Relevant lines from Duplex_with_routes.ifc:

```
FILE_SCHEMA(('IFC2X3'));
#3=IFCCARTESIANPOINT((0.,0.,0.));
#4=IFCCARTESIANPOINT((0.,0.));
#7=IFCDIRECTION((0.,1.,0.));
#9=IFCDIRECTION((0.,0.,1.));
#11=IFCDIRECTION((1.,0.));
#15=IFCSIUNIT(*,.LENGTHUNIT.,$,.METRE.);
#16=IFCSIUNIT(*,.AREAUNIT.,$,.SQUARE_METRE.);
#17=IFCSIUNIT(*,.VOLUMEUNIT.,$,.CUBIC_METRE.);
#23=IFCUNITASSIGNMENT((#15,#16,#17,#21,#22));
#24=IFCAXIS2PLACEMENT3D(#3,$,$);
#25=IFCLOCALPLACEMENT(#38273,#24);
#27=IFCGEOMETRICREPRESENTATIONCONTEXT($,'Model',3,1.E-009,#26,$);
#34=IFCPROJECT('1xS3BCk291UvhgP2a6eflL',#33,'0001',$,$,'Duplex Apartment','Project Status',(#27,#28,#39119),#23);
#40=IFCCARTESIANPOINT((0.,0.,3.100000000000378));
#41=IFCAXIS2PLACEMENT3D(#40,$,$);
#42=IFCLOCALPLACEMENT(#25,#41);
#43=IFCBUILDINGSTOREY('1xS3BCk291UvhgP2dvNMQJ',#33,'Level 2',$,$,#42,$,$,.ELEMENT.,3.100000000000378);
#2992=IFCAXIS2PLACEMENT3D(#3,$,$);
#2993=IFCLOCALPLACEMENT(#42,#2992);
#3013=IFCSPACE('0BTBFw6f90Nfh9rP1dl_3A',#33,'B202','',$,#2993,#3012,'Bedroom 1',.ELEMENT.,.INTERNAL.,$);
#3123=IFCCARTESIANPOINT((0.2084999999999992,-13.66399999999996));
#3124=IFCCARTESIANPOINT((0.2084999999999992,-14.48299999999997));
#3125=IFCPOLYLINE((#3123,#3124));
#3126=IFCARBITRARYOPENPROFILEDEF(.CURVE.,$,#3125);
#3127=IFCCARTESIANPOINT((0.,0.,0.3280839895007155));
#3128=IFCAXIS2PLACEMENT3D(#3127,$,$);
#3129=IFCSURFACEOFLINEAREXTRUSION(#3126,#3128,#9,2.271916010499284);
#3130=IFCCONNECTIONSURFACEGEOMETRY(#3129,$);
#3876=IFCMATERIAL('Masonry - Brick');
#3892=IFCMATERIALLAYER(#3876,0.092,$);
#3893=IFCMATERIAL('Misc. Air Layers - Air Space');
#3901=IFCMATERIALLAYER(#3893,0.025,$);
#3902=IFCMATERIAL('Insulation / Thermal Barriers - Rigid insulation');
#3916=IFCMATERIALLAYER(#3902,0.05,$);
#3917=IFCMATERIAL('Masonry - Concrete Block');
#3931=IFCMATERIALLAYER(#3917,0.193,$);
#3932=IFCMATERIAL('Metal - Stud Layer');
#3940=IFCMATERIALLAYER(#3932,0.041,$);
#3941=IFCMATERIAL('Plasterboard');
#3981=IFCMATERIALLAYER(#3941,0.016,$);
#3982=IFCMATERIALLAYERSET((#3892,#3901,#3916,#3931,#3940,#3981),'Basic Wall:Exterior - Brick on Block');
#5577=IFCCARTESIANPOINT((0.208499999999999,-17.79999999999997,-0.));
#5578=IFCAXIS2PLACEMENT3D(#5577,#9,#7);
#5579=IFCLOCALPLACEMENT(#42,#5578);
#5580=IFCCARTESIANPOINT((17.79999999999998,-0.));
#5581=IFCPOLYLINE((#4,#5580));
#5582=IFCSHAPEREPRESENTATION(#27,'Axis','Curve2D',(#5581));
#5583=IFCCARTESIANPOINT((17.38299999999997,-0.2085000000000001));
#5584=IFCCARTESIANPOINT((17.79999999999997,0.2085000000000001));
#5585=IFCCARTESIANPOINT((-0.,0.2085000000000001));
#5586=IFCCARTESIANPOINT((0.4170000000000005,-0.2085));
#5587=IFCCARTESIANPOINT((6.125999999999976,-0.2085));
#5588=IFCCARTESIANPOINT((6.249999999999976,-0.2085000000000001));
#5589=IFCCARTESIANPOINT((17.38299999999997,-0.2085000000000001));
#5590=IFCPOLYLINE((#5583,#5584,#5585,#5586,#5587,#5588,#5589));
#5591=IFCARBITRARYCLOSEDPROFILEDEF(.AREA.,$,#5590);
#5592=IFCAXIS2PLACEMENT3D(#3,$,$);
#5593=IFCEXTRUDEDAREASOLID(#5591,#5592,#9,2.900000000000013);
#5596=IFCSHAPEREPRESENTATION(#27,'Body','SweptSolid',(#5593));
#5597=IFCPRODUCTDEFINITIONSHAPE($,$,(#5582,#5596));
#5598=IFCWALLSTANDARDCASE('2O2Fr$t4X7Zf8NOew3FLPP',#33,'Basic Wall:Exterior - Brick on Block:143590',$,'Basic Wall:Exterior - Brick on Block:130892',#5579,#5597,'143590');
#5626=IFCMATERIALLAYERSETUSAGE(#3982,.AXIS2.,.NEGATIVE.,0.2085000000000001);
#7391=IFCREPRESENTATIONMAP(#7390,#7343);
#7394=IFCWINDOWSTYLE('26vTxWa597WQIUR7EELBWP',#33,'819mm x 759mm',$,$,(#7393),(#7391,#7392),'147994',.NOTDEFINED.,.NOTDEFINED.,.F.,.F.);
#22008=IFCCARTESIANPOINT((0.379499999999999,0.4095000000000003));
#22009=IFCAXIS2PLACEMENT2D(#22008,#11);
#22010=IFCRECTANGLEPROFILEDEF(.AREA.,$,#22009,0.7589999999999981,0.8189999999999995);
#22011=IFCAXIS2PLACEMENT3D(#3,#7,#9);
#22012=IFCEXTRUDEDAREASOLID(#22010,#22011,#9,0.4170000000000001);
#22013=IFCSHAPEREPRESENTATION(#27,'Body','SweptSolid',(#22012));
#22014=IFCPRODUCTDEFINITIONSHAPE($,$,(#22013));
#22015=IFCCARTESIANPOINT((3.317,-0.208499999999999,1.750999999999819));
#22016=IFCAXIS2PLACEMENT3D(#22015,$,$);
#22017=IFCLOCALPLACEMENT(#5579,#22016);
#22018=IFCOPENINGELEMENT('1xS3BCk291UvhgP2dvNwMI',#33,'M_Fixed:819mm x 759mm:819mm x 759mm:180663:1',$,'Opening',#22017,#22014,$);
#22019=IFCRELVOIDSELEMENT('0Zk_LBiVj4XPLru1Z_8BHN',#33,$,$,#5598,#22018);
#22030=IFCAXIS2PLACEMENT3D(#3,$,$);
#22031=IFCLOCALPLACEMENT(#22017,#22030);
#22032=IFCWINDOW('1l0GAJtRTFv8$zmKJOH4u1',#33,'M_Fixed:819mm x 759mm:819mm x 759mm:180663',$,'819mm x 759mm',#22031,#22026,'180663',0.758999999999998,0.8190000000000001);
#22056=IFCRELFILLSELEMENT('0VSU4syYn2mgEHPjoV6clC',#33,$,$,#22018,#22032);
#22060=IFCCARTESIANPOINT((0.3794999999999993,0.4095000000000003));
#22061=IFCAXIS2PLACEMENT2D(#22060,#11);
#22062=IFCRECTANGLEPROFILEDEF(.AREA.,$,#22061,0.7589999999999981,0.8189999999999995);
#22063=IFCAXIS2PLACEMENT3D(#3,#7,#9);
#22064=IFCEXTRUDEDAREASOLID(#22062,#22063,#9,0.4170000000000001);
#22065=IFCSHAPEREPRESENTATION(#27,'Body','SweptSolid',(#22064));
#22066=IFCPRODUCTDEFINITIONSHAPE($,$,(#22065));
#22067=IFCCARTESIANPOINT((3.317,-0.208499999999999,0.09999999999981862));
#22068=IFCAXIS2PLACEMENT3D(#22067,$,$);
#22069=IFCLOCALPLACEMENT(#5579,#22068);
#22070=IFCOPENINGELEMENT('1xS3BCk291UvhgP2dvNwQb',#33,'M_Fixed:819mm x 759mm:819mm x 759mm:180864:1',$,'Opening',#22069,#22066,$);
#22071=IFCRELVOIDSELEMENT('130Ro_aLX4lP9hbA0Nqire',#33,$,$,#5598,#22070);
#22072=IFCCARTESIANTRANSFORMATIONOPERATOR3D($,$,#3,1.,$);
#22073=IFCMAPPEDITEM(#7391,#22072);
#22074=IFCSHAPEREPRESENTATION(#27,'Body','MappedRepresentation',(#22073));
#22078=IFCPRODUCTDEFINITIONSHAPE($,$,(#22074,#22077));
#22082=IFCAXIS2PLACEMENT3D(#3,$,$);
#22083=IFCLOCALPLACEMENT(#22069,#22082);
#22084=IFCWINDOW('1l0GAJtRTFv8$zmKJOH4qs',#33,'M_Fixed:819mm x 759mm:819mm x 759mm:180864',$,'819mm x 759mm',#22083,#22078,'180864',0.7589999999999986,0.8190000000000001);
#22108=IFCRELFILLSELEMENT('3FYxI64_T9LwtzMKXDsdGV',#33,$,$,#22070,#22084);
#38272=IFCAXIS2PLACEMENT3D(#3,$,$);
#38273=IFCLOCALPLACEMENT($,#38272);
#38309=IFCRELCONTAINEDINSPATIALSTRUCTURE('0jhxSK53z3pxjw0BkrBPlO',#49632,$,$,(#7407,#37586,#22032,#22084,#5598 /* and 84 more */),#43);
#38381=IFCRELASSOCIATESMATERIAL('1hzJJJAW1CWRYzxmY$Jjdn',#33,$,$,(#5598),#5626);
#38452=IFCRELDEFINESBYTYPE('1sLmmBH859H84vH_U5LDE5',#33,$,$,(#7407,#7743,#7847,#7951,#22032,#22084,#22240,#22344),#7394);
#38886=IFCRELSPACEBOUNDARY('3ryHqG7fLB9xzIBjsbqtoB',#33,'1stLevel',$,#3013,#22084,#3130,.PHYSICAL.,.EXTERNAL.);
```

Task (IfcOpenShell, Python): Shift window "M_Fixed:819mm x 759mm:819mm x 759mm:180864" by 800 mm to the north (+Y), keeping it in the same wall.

```python
import numpy as np
import ifcopenshell
import ifcopenshell.api.geometry
import ifcopenshell.util.placement

model = ifcopenshell.open("Duplex_with_routes.ifc")

window = model.by_guid("1l0GAJtRTFv8$zmKJOH4qs")
opening = window.FillsVoids[0].RelatingOpeningElement
wall = opening.VoidsElements[0].RelatingBuildingElement

wall_matrix = ifcopenshell.util.placement.get_local_placement(wall.ObjectPlacement)
shift = wall_matrix[:3, 0] * 0.8
before = ifcopenshell.util.placement.get_local_placement(window.ObjectPlacement)[:3, 3].copy()

# The window is placed relative to its opening, so it follows when the opening moves.
matrix = ifcopenshell.util.placement.get_local_placement(opening.ObjectPlacement)
matrix[:3, 3] += shift
ifcopenshell.api.geometry.edit_object_placement(
    model, product=opening, matrix=matrix, is_si=False, should_transform_children=True
)

# Space boundary surfaces are stored in each space's coordinates; move them too.
for rel in window.ProvidesBoundaries:
    if not rel.ConnectionGeometry:
        continue
    surface = rel.ConnectionGeometry.SurfaceOnRelatingElement
    space_matrix = ifcopenshell.util.placement.get_local_placement(rel.RelatingSpace.ObjectPlacement)
    point = np.array(surface.Position.Location.Coordinates) + space_matrix[:3, :3].T @ shift
    surface.Position = model.createIfcAxis2Placement3D(
        model.createIfcCartesianPoint(point.tolist()), surface.Position.Axis, surface.Position.RefDirection
    )

after = ifcopenshell.util.placement.get_local_placement(window.ObjectPlacement)[:3, 3]
print("window moved by", (after - before).round(3) + 0.0)

model.write("Duplex_with_routes_updated.ifc")
```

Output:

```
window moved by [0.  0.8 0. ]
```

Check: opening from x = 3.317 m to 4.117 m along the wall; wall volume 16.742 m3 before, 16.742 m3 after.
